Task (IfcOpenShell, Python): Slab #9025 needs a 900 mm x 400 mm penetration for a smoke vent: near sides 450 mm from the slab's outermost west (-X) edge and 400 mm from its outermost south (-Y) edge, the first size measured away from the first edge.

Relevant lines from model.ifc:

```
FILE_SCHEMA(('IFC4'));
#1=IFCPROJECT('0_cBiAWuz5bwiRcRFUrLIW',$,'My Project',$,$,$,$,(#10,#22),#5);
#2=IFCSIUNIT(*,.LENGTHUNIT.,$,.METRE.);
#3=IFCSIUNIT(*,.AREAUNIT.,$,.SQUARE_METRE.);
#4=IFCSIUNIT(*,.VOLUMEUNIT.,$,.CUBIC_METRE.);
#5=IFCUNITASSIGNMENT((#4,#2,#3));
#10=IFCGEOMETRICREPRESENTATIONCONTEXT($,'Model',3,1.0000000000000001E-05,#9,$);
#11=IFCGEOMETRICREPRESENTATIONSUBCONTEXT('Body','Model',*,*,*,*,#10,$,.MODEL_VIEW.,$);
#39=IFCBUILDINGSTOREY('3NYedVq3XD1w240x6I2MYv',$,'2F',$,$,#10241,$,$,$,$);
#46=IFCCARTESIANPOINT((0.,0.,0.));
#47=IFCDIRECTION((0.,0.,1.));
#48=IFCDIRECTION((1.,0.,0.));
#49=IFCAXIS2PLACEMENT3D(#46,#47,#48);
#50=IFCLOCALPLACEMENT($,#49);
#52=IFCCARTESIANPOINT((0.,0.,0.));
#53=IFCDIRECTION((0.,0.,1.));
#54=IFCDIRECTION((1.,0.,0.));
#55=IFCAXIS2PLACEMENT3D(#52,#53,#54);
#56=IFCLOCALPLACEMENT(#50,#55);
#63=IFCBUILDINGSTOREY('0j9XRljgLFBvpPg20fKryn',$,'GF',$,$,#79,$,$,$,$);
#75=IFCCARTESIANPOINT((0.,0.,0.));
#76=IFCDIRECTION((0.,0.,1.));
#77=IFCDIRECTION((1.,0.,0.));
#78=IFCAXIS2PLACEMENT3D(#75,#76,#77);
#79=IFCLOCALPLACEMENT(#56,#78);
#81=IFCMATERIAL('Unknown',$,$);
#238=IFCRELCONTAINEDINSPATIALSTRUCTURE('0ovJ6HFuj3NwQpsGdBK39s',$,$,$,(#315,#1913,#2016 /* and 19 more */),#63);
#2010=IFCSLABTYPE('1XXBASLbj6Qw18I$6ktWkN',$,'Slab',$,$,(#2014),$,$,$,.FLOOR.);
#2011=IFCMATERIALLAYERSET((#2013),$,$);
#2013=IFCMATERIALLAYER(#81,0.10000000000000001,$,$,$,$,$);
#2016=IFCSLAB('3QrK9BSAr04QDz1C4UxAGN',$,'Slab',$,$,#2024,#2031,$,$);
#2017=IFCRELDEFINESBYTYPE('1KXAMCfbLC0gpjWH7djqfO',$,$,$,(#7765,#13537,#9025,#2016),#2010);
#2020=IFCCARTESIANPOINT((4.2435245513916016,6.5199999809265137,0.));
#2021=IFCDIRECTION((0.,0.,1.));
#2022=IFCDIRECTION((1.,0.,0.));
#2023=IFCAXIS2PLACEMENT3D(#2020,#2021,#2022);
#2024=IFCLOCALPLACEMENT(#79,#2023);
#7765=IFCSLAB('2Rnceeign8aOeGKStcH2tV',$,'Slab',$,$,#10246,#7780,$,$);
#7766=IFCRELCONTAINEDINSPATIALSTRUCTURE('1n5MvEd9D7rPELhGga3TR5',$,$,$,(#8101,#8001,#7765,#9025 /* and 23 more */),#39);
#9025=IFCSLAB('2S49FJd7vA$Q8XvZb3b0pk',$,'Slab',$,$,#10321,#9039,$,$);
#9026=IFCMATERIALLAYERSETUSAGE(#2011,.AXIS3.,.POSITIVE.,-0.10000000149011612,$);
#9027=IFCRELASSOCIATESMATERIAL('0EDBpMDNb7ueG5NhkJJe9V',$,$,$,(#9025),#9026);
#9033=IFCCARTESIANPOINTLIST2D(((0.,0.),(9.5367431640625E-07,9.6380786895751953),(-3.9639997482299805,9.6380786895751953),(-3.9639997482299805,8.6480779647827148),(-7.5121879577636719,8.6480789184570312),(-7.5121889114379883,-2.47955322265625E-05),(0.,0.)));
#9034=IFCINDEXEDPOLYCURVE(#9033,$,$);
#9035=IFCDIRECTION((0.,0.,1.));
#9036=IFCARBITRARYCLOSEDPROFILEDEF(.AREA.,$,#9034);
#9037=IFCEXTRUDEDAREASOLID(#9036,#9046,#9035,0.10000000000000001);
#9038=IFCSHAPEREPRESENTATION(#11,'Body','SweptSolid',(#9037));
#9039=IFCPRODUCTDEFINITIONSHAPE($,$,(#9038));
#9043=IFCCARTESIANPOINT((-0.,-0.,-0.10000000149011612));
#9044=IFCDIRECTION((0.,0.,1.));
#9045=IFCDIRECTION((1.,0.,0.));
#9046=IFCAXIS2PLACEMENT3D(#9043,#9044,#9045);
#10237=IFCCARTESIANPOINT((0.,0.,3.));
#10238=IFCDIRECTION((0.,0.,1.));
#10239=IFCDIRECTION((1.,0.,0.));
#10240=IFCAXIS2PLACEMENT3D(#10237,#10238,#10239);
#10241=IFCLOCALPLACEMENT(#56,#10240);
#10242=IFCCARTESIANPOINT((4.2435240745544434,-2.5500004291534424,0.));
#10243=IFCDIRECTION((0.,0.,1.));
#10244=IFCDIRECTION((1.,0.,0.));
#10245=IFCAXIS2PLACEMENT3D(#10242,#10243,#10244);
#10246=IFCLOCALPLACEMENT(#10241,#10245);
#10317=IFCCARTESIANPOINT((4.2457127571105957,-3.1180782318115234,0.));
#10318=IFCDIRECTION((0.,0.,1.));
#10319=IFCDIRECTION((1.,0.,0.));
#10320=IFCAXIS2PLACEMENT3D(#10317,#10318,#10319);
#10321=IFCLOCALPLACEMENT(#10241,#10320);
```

```python
import numpy as np
import ifcopenshell
import ifcopenshell.api.feature
import ifcopenshell.api.geometry
import ifcopenshell.api.root
import ifcopenshell.geom
import ifcopenshell.util.placement
import ifcopenshell.util.representation
import ifcopenshell.util.shape
import ifcopenshell.util.unit

model = ifcopenshell.open("model.ifc")
unit_scale = ifcopenshell.util.unit.calculate_unit_scale(model)
settings = ifcopenshell.geom.settings()


def volume(element):
    """Net volume in cubic metres, openings subtracted."""
    shape = ifcopenshell.geom.create_shape(settings, element)
    return ifcopenshell.util.shape.get_volume(shape.geometry)


slab = model.by_guid("2S49FJd7vA$Q8XvZb3b0pk")
before = volume(slab)

# Extent in the slab's own axes, in metres. The edges named are its -X and -Y sides.
slab_shape = ifcopenshell.geom.create_shape(settings, slab)
vertices = ifcopenshell.util.shape.get_vertices(slab_shape.geometry)
x_min, y_min, bottom = vertices.min(axis=0)
top = vertices[:, 2].max()

opening = ifcopenshell.api.root.create_entity(model, ifc_class="IfcOpeningElement", name="Smoke vent opening", predefined_type="OPENING")
context = ifcopenshell.util.representation.get_context(model, "Model", "Body", "MODEL_VIEW")
width, depth = 0.9, 0.4
outline = [(0.0, 0.0), (width, 0.0), (width, depth), (0.0, depth), (0.0, 0.0)]
# Overshoot both faces by 50 mm so the cut is clean.
shape = ifcopenshell.api.geometry.add_slab_representation(
    model, context=context, depth=top - bottom + 0.1, polyline=outline
)
ifcopenshell.api.geometry.assign_representation(model, product=opening, representation=shape)

matrix = ifcopenshell.util.placement.get_local_placement(slab.ObjectPlacement)
matrix[:, 3] = matrix @ np.append(np.array([x_min + 0.45, y_min + 0.4, bottom - 0.05]) / unit_scale, 1.0)
ifcopenshell.api.geometry.edit_object_placement(model, product=opening, matrix=matrix, is_si=False)
ifcopenshell.api.feature.add_feature(model, feature=opening, element=slab)

after = volume(slab)

print(f"slab volume {before:.3f} -> {after:.3f} m3")

model.write("model-out.ifc")
```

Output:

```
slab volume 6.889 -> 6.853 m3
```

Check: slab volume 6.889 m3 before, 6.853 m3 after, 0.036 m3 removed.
